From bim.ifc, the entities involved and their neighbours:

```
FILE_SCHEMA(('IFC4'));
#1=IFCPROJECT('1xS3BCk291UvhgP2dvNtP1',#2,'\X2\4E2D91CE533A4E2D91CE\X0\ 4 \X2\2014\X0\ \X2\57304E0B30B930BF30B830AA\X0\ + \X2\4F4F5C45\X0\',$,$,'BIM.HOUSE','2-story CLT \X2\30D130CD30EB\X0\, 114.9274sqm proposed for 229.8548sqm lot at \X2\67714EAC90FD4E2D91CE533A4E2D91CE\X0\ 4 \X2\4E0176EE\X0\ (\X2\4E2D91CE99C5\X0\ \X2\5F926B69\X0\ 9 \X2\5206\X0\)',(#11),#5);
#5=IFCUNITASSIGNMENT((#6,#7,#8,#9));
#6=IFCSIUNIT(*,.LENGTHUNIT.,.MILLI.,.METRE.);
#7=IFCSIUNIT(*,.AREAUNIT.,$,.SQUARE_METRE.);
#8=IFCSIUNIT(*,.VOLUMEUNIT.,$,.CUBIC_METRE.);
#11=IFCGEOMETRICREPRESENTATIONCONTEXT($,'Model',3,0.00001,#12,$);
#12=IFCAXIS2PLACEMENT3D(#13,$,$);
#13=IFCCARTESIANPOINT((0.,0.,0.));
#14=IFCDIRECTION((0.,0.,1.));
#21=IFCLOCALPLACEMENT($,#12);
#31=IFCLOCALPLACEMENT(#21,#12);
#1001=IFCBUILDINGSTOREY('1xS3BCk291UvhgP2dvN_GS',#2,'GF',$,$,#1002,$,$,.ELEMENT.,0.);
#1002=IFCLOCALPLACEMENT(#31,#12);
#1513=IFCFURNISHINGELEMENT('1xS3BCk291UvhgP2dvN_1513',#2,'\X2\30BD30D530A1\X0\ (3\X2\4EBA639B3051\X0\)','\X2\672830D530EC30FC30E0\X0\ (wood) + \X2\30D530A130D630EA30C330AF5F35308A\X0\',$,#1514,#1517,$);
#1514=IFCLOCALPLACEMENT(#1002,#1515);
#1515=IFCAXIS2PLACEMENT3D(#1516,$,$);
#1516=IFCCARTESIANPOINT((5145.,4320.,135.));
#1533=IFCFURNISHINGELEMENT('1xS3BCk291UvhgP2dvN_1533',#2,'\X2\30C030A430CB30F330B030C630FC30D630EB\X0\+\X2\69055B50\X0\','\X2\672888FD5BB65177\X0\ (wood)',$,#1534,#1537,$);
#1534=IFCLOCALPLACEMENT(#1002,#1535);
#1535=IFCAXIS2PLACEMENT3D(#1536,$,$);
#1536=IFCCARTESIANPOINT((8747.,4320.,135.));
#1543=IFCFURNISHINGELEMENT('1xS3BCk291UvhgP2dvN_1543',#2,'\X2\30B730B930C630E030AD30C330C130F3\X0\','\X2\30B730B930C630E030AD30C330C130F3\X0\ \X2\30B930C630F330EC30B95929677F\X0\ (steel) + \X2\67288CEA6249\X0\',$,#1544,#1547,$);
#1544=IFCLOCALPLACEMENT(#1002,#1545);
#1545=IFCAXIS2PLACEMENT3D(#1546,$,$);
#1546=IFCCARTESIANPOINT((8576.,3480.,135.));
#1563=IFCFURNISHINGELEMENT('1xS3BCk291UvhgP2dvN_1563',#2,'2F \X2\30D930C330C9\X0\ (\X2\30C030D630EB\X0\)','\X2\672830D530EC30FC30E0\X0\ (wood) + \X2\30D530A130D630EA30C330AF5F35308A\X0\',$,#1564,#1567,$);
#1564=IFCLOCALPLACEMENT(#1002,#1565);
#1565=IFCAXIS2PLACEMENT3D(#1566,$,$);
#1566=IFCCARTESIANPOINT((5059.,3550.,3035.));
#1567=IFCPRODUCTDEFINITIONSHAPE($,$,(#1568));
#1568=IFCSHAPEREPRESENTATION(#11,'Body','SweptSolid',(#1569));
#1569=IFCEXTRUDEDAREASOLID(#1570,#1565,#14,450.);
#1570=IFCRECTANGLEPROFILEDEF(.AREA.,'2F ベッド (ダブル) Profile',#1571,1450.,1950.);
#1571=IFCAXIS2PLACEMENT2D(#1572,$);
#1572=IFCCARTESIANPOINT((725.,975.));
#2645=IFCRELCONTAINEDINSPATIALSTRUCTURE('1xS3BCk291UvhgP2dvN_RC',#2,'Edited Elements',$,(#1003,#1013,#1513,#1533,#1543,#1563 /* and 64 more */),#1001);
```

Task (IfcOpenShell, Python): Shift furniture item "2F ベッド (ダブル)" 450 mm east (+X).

```python
import ifcopenshell
import ifcopenshell.api.geometry
import ifcopenshell.util.placement

model = ifcopenshell.open("bim.ifc")

item = model.by_guid("1xS3BCk291UvhgP2dvN_1563")
matrix = ifcopenshell.util.placement.get_local_placement(item.ObjectPlacement)
matrix[0, 3] += 450.0
ifcopenshell.api.geometry.edit_object_placement(model, product=item, matrix=matrix, is_si=False)

print(ifcopenshell.util.placement.get_local_placement(item.ObjectPlacement).round(3) + 0.0)

model.write("bim_updated.ifc")
```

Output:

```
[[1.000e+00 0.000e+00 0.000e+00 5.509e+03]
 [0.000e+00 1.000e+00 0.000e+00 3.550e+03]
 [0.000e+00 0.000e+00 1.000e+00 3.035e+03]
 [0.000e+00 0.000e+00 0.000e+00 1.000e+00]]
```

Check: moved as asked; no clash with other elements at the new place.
